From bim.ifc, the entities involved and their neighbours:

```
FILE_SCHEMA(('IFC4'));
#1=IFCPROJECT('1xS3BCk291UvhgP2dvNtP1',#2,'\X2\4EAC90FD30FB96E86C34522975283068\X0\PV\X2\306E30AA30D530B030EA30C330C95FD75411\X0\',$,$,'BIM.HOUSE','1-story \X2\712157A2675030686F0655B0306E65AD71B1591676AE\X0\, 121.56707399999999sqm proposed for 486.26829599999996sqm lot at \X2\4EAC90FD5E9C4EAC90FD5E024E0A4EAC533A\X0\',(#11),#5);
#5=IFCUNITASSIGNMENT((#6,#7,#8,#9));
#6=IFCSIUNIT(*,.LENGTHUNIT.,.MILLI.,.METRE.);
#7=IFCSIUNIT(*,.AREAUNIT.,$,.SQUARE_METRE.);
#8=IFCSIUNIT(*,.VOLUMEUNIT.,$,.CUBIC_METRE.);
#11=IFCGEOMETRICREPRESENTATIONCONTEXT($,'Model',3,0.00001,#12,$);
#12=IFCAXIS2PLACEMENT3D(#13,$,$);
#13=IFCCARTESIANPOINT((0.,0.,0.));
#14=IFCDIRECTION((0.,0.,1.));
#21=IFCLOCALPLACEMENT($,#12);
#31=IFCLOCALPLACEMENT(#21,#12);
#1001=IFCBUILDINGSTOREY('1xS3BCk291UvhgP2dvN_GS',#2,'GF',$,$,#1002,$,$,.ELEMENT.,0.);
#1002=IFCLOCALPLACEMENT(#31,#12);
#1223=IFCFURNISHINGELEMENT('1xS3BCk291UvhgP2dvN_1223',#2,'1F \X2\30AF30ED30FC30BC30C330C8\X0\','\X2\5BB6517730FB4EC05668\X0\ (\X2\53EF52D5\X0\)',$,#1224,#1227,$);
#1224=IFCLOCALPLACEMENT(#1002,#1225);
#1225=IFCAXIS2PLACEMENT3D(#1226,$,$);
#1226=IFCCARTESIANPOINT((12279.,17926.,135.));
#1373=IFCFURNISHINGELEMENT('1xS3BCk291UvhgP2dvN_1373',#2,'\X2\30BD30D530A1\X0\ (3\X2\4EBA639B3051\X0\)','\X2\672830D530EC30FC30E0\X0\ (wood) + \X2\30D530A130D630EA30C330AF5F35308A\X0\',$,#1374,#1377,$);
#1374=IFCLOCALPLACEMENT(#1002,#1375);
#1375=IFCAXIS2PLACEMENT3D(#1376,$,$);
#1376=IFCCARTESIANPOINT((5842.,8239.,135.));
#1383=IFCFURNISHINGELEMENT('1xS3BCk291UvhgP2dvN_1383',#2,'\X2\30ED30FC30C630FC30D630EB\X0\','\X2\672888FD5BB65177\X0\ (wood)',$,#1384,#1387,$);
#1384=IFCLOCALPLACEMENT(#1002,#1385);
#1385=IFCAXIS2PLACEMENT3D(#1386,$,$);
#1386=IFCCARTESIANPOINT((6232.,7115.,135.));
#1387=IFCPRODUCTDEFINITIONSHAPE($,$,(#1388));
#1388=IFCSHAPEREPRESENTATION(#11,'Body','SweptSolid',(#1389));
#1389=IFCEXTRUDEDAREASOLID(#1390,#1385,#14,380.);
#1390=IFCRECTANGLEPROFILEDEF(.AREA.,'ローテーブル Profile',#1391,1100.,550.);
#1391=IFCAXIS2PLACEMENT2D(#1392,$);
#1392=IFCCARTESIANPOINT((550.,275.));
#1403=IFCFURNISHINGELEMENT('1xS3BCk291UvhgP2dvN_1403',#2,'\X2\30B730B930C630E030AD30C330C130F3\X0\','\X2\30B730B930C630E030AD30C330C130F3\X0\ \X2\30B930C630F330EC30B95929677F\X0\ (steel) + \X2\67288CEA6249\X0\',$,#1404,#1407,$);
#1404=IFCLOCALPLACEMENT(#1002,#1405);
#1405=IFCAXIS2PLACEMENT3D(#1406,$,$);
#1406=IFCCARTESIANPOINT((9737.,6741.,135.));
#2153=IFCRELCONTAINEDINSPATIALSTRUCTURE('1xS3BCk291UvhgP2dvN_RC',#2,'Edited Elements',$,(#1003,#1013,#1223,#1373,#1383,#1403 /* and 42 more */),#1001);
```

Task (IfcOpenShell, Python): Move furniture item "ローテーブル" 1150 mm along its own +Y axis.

```python
import ifcopenshell
import ifcopenshell.api.geometry
import ifcopenshell.util.placement
import ifcopenshell.util.unit

model = ifcopenshell.open("bim.ifc")
unit_scale = ifcopenshell.util.unit.calculate_unit_scale(model)

item = model.by_guid("1xS3BCk291UvhgP2dvN_1383")
matrix = ifcopenshell.util.placement.get_local_placement(item.ObjectPlacement)
matrix[:3, 3] += matrix[:3, 1] * 1.15 / unit_scale
ifcopenshell.api.geometry.edit_object_placement(model, product=item, matrix=matrix, is_si=False)

print(ifcopenshell.util.placement.get_local_placement(item.ObjectPlacement).round(3) + 0.0)

model.write("bim_rev.ifc")
```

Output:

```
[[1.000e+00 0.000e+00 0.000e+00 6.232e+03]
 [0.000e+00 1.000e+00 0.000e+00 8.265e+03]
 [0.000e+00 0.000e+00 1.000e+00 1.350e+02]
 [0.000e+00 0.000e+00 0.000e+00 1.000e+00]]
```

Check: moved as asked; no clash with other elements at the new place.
